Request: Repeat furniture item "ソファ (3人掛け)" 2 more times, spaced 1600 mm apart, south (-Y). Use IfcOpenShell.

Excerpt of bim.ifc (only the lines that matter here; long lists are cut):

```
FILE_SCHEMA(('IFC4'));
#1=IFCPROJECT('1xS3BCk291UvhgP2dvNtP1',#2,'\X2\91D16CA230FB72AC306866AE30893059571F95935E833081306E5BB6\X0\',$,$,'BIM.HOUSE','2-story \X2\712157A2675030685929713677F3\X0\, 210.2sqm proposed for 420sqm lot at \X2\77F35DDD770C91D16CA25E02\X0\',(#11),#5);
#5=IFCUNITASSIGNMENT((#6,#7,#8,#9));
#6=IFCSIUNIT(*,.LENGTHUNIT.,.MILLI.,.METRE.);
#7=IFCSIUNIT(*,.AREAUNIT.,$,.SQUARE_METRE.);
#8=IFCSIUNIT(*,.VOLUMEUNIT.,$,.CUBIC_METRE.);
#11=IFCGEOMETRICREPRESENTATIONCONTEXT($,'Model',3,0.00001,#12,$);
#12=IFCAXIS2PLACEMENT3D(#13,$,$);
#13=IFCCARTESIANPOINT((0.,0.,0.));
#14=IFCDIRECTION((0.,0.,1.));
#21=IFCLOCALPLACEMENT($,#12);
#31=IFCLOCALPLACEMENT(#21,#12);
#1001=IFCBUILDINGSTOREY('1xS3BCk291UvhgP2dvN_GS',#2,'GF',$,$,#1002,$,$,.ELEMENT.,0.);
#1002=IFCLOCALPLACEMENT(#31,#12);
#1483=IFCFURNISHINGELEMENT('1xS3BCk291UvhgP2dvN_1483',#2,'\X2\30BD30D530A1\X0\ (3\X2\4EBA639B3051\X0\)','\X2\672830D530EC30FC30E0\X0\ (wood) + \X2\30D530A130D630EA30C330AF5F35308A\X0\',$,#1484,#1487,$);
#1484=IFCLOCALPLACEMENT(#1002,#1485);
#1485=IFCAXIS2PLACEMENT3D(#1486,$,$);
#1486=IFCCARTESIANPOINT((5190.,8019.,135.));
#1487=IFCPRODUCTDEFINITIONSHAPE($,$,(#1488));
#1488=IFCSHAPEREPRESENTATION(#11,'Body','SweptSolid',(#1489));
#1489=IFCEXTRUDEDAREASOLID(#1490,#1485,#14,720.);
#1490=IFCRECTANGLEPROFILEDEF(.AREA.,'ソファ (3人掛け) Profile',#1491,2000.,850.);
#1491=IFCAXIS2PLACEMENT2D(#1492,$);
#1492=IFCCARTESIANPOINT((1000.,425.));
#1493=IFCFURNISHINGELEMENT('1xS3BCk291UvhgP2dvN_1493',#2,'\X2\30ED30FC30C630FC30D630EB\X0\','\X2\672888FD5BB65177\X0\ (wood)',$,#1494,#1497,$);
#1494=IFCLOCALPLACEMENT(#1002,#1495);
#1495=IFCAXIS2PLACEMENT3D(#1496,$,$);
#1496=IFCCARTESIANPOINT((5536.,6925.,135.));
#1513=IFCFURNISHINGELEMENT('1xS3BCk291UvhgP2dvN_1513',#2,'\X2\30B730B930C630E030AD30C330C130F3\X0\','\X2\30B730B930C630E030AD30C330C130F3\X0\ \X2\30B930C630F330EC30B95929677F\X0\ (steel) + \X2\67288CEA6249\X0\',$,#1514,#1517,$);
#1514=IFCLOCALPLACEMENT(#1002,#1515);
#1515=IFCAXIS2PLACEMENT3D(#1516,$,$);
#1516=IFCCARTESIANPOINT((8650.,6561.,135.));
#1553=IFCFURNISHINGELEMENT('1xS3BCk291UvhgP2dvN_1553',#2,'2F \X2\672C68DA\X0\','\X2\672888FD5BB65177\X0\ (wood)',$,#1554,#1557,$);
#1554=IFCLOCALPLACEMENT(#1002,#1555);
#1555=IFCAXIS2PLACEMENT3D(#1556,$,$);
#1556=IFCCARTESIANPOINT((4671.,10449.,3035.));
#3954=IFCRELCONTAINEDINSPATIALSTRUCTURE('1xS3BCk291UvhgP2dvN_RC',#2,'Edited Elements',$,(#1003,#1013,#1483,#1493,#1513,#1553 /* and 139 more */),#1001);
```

```python
import numpy as np
import ifcopenshell
import ifcopenshell.api.geometry
import ifcopenshell.api.root
import ifcopenshell.util.element
import ifcopenshell.util.placement
import ifcopenshell.util.unit

model = ifcopenshell.open("bim.ifc")
unit_scale = ifcopenshell.util.unit.calculate_unit_scale(model)


def reuse_history(source, copy):
    """copy_class also copies each property set's owner history, people and application; keep the originals."""
    for rel in copy.IsDefinedBy:
        if rel.is_a("IfcRelDefinesByProperties") and (history := rel.RelatingPropertyDefinition.OwnerHistory):
            rel.RelatingPropertyDefinition.OwnerHistory = source.OwnerHistory
            ifcopenshell.util.element.remove_deep2(model, history)


source = model.by_guid("1xS3BCk291UvhgP2dvN_1483")
base = ifcopenshell.util.placement.get_local_placement(source.ObjectPlacement)
step = np.array([0.0, -1.0, 0.0]) * 1.6 / unit_scale

for i in range(1, 3):
    copy = ifcopenshell.api.root.copy_class(model, product=source)
    copy.Representation = ifcopenshell.util.element.copy_deep(
        model, source.Representation, exclude=["IfcGeometricRepresentationContext", "IfcRepresentationMap"]
    )
    reuse_history(source, copy)
    matrix = base.copy()
    matrix[:3, 3] += i * step
    print("added at", matrix[:3, 3].round(3) + 0.0)
    ifcopenshell.api.geometry.edit_object_placement(model, product=copy, matrix=matrix, is_si=False)

model.write("bim_v2.ifc")
```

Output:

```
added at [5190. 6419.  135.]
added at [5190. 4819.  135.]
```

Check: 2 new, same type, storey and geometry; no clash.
